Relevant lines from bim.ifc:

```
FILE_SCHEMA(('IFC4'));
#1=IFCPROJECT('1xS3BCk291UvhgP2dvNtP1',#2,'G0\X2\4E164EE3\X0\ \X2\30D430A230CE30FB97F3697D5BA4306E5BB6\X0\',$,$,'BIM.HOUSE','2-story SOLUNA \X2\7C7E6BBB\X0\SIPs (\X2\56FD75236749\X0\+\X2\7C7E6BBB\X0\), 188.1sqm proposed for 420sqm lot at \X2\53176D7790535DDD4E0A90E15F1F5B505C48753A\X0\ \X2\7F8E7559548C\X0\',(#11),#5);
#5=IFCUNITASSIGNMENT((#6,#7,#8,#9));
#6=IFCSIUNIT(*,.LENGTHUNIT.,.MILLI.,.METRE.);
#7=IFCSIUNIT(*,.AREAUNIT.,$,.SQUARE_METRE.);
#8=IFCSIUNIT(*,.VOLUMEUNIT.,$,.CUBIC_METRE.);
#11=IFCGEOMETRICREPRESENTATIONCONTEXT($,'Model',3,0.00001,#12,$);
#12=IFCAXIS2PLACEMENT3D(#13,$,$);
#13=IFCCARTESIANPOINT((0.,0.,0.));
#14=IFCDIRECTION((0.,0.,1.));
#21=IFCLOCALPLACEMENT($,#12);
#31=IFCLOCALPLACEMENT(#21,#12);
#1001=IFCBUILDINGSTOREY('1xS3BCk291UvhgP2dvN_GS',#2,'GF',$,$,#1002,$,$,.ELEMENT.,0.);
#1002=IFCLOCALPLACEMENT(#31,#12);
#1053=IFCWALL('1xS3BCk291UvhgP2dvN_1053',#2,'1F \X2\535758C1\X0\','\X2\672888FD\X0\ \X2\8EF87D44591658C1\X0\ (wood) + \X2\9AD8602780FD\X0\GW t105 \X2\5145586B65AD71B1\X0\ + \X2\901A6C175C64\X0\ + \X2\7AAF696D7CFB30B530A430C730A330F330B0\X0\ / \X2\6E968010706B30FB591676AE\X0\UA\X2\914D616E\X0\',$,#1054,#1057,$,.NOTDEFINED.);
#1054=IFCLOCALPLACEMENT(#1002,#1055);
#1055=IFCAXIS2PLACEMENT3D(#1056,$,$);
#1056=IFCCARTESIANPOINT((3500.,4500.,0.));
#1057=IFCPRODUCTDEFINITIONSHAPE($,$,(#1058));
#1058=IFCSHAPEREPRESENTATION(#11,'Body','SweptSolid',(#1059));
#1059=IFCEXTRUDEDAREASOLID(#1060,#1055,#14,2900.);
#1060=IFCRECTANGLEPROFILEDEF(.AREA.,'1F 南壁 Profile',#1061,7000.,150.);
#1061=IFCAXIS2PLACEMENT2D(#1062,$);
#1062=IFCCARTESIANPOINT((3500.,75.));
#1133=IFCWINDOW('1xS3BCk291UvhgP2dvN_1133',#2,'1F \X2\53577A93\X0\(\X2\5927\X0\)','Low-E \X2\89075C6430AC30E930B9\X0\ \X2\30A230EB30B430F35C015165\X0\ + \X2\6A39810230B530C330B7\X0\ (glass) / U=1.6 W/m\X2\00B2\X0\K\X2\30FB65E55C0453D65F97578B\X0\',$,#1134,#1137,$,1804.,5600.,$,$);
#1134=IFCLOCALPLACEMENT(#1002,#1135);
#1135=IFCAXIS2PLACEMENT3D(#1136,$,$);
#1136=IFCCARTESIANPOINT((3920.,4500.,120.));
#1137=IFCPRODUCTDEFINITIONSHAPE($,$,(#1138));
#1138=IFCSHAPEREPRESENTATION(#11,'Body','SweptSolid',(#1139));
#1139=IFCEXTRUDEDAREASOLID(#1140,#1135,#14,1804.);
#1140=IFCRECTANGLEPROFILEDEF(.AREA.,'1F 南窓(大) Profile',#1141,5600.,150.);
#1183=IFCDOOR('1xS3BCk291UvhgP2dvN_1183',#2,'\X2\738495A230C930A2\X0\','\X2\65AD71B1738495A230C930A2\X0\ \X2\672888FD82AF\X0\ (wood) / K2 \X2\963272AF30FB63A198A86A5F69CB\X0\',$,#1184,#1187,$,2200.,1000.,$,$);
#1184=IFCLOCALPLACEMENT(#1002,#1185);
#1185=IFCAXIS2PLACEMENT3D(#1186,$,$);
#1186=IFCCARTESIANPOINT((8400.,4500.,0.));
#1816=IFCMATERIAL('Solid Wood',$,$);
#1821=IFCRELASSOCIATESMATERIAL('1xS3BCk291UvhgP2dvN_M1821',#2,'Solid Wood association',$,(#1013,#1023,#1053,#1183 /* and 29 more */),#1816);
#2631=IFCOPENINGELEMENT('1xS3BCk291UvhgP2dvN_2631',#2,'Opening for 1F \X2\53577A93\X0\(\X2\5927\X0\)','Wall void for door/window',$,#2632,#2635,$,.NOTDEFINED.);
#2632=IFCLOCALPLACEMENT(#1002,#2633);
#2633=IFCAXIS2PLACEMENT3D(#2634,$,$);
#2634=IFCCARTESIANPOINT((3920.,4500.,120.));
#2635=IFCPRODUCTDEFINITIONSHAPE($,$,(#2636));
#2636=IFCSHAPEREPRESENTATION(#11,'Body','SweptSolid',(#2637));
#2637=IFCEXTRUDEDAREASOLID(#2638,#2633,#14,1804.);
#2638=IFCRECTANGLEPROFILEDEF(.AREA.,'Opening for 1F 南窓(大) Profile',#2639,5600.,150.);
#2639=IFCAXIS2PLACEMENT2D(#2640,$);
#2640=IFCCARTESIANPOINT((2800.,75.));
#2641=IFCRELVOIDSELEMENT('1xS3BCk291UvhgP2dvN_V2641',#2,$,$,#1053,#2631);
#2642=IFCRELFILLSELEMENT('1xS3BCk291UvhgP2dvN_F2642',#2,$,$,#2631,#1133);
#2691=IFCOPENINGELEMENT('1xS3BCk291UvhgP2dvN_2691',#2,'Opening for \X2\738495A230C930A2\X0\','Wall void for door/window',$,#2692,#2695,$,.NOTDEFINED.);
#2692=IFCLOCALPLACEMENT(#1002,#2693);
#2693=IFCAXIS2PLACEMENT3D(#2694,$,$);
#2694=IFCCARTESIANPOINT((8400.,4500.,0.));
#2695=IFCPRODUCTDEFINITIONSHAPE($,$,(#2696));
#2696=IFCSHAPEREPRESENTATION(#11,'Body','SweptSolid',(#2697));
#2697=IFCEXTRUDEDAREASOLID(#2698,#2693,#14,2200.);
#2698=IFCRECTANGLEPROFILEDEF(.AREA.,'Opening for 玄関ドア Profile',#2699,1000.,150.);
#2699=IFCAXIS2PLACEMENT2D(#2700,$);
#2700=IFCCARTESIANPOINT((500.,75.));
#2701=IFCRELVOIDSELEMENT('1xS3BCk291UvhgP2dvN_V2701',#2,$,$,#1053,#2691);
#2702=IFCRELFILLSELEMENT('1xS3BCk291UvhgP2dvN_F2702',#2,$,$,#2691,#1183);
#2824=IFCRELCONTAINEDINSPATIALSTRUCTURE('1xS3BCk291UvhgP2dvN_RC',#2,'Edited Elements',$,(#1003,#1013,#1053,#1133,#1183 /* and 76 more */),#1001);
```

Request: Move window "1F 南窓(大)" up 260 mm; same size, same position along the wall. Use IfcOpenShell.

```python
import numpy as np
import ifcopenshell
import ifcopenshell.api.geometry
import ifcopenshell.util.placement
import ifcopenshell.util.unit

model = ifcopenshell.open("bim.ifc")
unit_scale = ifcopenshell.util.unit.calculate_unit_scale(model)

window = model.by_guid("1xS3BCk291UvhgP2dvN_1133")
opening = window.FillsVoids[0].RelatingOpeningElement
dz = 0.26 / unit_scale

shift = np.array([0.0, 0.0, dz])
# The window is not placed relative to its opening, so move both.
for product in (opening, window):
    matrix = ifcopenshell.util.placement.get_local_placement(product.ObjectPlacement)
    matrix[:3, 3] += shift
    ifcopenshell.api.geometry.edit_object_placement(model, product=product, matrix=matrix, is_si=False)

print(f"moved by {dz * unit_scale:+.3f} m")

model.write("bim_rev.ifc")
```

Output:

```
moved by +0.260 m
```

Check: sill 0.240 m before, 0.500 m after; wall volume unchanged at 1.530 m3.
